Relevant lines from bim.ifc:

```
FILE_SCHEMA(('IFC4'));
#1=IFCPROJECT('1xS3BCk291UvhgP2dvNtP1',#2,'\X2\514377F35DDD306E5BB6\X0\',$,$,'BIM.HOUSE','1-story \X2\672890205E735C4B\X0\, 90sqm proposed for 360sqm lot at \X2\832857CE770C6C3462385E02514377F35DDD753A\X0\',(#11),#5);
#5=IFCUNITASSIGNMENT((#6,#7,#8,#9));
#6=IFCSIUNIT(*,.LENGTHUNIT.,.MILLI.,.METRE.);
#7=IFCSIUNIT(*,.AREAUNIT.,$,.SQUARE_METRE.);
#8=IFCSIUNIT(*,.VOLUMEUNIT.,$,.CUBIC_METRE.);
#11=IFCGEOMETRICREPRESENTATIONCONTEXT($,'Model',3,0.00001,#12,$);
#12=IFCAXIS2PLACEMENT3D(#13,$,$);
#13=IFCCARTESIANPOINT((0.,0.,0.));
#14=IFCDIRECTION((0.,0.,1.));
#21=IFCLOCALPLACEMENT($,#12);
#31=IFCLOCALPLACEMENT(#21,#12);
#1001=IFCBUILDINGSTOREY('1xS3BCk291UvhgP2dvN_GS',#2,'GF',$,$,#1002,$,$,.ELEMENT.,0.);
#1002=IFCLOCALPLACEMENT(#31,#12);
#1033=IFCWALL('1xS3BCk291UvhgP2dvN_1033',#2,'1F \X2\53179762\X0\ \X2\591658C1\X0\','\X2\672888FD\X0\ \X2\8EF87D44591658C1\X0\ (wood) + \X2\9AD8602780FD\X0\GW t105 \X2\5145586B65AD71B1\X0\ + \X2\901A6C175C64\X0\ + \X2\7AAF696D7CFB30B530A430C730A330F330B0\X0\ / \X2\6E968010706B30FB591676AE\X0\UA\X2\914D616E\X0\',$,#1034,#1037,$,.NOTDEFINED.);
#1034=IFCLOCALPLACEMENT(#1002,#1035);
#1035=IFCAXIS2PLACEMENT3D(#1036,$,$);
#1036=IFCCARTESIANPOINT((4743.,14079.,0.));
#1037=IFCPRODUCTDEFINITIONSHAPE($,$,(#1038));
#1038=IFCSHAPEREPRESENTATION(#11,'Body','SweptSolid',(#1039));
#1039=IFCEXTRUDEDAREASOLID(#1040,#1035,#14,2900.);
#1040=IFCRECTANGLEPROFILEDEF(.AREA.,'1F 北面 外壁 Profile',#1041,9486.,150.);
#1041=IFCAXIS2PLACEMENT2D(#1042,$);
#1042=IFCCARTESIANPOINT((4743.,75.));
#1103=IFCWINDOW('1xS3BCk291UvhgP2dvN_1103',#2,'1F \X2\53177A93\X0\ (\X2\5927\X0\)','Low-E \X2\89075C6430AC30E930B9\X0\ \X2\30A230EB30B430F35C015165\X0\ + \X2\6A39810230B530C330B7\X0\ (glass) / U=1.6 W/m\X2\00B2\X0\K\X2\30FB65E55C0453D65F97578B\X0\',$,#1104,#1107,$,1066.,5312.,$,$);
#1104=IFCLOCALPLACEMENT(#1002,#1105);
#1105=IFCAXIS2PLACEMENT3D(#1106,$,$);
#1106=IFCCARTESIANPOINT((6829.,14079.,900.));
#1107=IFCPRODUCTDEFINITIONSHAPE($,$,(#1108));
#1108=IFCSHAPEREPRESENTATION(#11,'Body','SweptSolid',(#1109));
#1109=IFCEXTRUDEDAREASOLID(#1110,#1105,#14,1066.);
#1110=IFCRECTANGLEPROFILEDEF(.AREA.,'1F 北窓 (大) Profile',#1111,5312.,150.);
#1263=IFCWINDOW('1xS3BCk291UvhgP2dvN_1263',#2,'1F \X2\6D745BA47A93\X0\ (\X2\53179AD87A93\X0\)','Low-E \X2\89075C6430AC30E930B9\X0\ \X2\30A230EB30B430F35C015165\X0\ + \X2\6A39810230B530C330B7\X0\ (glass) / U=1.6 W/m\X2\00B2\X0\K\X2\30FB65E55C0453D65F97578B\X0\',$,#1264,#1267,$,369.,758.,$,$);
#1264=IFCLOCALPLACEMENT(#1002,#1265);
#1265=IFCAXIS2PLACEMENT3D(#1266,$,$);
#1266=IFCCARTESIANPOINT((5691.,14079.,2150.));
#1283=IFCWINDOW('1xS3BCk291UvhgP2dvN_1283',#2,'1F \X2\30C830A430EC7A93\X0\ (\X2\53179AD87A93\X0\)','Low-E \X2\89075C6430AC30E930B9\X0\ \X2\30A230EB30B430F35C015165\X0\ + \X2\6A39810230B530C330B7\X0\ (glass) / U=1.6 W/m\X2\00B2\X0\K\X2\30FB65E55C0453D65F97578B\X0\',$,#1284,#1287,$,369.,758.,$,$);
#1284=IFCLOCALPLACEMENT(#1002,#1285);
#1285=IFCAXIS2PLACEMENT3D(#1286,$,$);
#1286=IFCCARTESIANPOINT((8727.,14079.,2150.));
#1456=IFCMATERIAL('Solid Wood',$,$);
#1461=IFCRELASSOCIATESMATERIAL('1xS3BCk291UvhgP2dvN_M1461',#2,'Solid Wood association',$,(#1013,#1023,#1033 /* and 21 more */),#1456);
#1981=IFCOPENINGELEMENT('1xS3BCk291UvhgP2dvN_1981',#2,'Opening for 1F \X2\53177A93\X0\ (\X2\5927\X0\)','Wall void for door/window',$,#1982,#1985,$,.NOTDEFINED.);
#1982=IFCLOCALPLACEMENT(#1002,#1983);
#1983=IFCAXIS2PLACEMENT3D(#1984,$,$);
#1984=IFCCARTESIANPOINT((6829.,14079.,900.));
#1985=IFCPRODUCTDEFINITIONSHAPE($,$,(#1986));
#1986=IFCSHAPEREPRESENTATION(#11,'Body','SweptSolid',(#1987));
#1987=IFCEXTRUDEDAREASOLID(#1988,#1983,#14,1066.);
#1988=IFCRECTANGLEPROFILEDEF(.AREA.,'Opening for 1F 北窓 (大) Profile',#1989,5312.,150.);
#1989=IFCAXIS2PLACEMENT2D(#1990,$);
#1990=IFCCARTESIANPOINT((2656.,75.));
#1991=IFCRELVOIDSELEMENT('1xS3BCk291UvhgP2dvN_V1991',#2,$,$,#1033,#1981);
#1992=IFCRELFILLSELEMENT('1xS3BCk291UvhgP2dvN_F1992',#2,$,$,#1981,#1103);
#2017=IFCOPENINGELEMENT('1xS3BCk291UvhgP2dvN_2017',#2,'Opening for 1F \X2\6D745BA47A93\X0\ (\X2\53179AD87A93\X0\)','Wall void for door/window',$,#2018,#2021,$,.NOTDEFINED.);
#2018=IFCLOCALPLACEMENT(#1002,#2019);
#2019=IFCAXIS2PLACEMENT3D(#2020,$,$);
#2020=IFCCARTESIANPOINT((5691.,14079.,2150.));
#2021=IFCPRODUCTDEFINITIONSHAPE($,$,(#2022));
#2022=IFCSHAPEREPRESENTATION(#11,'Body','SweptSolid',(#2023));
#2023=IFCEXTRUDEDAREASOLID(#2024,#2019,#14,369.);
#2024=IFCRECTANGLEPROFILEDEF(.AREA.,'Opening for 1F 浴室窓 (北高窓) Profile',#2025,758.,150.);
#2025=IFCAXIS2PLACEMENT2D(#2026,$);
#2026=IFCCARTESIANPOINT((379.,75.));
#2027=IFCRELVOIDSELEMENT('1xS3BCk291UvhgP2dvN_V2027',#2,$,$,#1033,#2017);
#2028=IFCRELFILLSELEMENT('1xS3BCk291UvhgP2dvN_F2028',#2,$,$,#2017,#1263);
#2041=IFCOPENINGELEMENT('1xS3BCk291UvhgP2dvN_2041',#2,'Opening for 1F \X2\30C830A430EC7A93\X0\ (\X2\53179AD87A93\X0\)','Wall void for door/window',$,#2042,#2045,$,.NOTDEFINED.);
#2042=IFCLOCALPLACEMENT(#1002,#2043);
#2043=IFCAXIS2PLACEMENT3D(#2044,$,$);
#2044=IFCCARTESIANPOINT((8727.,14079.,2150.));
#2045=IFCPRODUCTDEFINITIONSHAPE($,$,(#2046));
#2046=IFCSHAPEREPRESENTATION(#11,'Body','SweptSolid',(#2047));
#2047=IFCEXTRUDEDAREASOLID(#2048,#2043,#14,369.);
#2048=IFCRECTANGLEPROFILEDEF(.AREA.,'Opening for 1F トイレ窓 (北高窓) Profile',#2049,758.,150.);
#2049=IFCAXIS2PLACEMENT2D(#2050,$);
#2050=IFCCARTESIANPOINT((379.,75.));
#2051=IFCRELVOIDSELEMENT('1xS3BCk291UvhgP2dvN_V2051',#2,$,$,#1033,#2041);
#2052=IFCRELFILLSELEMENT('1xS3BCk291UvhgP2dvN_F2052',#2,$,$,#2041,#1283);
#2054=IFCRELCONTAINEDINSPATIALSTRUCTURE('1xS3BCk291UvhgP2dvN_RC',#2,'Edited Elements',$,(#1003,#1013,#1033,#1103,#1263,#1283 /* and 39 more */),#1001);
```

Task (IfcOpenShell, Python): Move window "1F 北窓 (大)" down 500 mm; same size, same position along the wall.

```python
import numpy as np
import ifcopenshell
import ifcopenshell.api.geometry
import ifcopenshell.util.placement
import ifcopenshell.util.unit

model = ifcopenshell.open("bim.ifc")
unit_scale = ifcopenshell.util.unit.calculate_unit_scale(model)

window = model.by_guid("1xS3BCk291UvhgP2dvN_1103")
opening = window.FillsVoids[0].RelatingOpeningElement
dz = -500.0

shift = np.array([0.0, 0.0, dz])
# The window is not placed relative to its opening, so move both.
for product in (opening, window):
    matrix = ifcopenshell.util.placement.get_local_placement(product.ObjectPlacement)
    matrix[:3, 3] += shift
    ifcopenshell.api.geometry.edit_object_placement(model, product=product, matrix=matrix, is_si=False)

print(f"moved by {dz * unit_scale:+.3f} m")

model.write("bim_v2.ifc")
```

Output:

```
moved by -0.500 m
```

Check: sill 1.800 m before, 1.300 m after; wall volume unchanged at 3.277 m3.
